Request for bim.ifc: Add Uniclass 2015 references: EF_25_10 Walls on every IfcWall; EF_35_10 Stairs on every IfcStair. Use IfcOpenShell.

First a look at what the model holds.

```python
import ifcopenshell

model = ifcopenshell.open("bim.ifc")
print(model.schema)
print("classifications:", [c.Name for c in model.by_type("IfcClassification")])
for ifc_class in ("IfcDoor", "IfcRoof", "IfcStair", "IfcWall", "IfcWindow"):
    print(ifc_class, len(model.by_type(ifc_class)))
```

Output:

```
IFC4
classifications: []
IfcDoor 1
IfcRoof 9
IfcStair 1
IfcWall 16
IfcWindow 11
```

```python
import ifcopenshell
import ifcopenshell.api.classification

model = ifcopenshell.open("bim.ifc")

system = ifcopenshell.api.classification.add_classification(model, classification="Uniclass 2015")

codes = {
    "IfcWall": ("EF_25_10", "Walls"),
    "IfcStair": ("EF_35_10", "Stairs"),
}
for ifc_class, (code, name) in codes.items():
    products = model.by_type(ifc_class)
    ifcopenshell.api.classification.add_reference(
        model, products=products, classification=system, identification=code, name=name
    )
    print(code, len(products))

model.write("bim_updated.ifc")
```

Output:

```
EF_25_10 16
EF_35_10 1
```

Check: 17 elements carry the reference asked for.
